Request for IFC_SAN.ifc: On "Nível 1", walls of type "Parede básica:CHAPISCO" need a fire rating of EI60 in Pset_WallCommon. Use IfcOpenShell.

First a look at what the model holds.

```python
import ifcopenshell
import ifcopenshell.util.element

model = ifcopenshell.open("IFC_SAN.ifc")
print(model.schema)
storey = next(s for s in model.by_type("IfcBuildingStorey") if s.Name == "Nível 1")
walls = [e for e in ifcopenshell.util.element.get_decomposition(storey) if e.is_a("IfcWall")]
seen = {}
for e in walls:
    element_type = ifcopenshell.util.element.get_type(e)
    key = (element_type.Name if element_type != e and element_type else None, ifcopenshell.util.element.get_pset(e, "Pset_WallCommon", "FireRating"))
    seen[key] = seen.get(key, 0) + 1
for (name, value), count in sorted(seen.items(), key=str):
    print(count, "x", name, "|", value)
```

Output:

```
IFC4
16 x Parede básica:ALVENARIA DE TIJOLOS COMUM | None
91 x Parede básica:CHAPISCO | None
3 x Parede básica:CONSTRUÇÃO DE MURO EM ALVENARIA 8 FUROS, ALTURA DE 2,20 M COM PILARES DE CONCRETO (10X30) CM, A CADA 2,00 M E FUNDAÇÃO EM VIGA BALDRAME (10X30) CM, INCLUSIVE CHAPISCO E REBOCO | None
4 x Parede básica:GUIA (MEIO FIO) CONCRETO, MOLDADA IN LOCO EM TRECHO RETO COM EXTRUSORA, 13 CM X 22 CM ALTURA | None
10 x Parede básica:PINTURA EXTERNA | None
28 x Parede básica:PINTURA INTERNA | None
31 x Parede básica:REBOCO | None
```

```python
import ifcopenshell
import ifcopenshell.api.pset
import ifcopenshell.util.element

model = ifcopenshell.open("IFC_SAN.ifc")

storey = next(s for s in model.by_type("IfcBuildingStorey") if s.Name == "Nível 1")
walls = [e for e in ifcopenshell.util.element.get_decomposition(storey) if e.is_a("IfcWall")]

count = 0
for e in walls:
    element_type = ifcopenshell.util.element.get_type(e)
    if element_type in (None, e) or element_type.Name != "Parede básica:CHAPISCO":
        continue
    # add_pset returns the element's existing set when there is one.
    pset = ifcopenshell.api.pset.add_pset(model, product=e, name="Pset_WallCommon")
    ifcopenshell.api.pset.edit_pset(model, pset=pset, properties={"FireRating": "EI60"})
    count += 1

print(count, "walls updated")

model.write("IFC_SAN_edited.ifc")
```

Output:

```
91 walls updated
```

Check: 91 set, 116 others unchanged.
